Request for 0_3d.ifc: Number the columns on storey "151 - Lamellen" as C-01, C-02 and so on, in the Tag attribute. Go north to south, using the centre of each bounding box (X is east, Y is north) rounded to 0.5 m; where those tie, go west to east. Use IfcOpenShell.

First a look at what the model holds.

```python
import ifcopenshell
import ifcopenshell.util.element
import ifcopenshell.util.placement

model = ifcopenshell.open("0_3d.ifc")
print(model.schema)
storey = next(s for s in model.by_type("IfcBuildingStorey") if s.Name == "151 - Lamellen")
columns = [e for e in ifcopenshell.util.element.get_decomposition(storey) if e.is_a("IfcColumn")]
for e in sorted(columns, key=lambda e: e.id()):
    origin = ifcopenshell.util.placement.get_local_placement(e.ObjectPlacement)[:3, 3]
    print(e.id(), e.Tag, e.Name, origin.round(2) + 0.0, sep=" | ")
```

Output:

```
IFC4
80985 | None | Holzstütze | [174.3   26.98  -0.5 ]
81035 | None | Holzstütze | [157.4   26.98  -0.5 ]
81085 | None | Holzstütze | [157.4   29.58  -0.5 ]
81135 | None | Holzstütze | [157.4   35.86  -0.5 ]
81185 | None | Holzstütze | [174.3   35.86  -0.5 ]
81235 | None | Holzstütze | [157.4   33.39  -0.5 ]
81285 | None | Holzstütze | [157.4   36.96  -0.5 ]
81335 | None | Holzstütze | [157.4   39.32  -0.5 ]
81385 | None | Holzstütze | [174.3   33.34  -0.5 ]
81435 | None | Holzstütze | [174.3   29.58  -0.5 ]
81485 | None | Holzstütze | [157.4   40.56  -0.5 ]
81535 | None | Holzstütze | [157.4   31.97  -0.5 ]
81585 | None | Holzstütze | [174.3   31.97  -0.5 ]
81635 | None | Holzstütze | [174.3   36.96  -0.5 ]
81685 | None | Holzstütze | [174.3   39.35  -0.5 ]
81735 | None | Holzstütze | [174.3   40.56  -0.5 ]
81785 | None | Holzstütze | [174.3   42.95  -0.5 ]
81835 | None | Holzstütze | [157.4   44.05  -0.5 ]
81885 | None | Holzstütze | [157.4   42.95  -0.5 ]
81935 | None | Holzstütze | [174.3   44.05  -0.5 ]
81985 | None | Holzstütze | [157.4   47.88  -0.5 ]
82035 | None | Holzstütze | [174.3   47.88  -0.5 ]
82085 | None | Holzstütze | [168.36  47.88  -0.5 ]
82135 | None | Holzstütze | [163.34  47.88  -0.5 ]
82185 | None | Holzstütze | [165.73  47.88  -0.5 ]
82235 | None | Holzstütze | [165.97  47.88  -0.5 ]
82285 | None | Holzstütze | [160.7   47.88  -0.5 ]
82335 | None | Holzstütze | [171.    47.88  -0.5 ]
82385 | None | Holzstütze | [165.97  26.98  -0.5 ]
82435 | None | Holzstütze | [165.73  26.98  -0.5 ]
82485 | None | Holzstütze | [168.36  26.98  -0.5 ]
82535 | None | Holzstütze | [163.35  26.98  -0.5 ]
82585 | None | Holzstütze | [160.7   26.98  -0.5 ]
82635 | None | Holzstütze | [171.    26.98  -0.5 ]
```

```python
import ifcopenshell
import ifcopenshell.geom
import ifcopenshell.util.element
import ifcopenshell.util.shape

model = ifcopenshell.open("0_3d.ifc")
settings = ifcopenshell.geom.settings()
settings.set("use-world-coords", True)


def centre(element):
    shape = ifcopenshell.geom.create_shape(settings, element)
    return ifcopenshell.util.shape.get_bbox_centroid(shape.geometry)


storey = next(s for s in model.by_type("IfcBuildingStorey") if s.Name == "151 - Lamellen")
columns = [e for e in ifcopenshell.util.element.get_decomposition(storey) if e.is_a("IfcColumn")]

# Insertion points can sit at a corner or the storey origin, so sort by the geometry (in metres).
centres = {e: centre(e) for e in columns}
columns.sort(key=lambda e: (-round(centres[e][1] / 0.5), centres[e][0]))

for i, e in enumerate(columns, start=1):
    number = f"C-{i:02d}"
    e.Tag = number
    print(e.id(), number)

model.write("0_3d_updated.ifc")
```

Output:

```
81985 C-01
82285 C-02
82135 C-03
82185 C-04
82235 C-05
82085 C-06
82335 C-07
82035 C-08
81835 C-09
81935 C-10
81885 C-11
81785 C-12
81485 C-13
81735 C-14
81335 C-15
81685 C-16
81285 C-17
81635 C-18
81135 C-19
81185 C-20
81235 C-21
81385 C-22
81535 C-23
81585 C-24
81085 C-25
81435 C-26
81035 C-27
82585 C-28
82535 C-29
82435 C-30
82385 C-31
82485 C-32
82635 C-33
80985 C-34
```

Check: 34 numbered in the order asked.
